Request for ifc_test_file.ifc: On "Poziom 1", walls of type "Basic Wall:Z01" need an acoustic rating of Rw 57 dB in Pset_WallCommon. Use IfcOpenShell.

First a look at what the model holds.

```python
import ifcopenshell
import ifcopenshell.util.element

model = ifcopenshell.open("ifc_test_file.ifc")
print(model.schema)
storey = next(s for s in model.by_type("IfcBuildingStorey") if s.Name == "Poziom 1")
walls = [e for e in ifcopenshell.util.element.get_decomposition(storey) if e.is_a("IfcWall")]
seen = {}
for e in walls:
    element_type = ifcopenshell.util.element.get_type(e)
    key = (element_type.Name if element_type != e and element_type else None, ifcopenshell.util.element.get_pset(e, "Pset_WallCommon", "AcousticRating"))
    seen[key] = seen.get(key, 0) + 1
for (name, value), count in sorted(seen.items(), key=str):
    print(count, "x", name, "|", value)
```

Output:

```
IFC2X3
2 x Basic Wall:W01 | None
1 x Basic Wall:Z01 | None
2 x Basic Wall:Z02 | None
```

```python
import ifcopenshell
import ifcopenshell.api.pset
import ifcopenshell.util.element

model = ifcopenshell.open("ifc_test_file.ifc")

storey = next(s for s in model.by_type("IfcBuildingStorey") if s.Name == "Poziom 1")
walls = [e for e in ifcopenshell.util.element.get_decomposition(storey) if e.is_a("IfcWall")]

count = 0
for e in walls:
    element_type = ifcopenshell.util.element.get_type(e)
    if element_type in (None, e) or element_type.Name != "Basic Wall:Z01":
        continue
    # add_pset returns the element's existing set when there is one.
    pset = ifcopenshell.api.pset.add_pset(model, product=e, name="Pset_WallCommon")
    ifcopenshell.api.pset.edit_pset(model, pset=pset, properties={"AcousticRating": "Rw 57 dB"})
    count += 1

print(count, "walls updated")

model.write("ifc_test_file_v2.ifc")
```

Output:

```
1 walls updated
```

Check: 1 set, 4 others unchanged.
